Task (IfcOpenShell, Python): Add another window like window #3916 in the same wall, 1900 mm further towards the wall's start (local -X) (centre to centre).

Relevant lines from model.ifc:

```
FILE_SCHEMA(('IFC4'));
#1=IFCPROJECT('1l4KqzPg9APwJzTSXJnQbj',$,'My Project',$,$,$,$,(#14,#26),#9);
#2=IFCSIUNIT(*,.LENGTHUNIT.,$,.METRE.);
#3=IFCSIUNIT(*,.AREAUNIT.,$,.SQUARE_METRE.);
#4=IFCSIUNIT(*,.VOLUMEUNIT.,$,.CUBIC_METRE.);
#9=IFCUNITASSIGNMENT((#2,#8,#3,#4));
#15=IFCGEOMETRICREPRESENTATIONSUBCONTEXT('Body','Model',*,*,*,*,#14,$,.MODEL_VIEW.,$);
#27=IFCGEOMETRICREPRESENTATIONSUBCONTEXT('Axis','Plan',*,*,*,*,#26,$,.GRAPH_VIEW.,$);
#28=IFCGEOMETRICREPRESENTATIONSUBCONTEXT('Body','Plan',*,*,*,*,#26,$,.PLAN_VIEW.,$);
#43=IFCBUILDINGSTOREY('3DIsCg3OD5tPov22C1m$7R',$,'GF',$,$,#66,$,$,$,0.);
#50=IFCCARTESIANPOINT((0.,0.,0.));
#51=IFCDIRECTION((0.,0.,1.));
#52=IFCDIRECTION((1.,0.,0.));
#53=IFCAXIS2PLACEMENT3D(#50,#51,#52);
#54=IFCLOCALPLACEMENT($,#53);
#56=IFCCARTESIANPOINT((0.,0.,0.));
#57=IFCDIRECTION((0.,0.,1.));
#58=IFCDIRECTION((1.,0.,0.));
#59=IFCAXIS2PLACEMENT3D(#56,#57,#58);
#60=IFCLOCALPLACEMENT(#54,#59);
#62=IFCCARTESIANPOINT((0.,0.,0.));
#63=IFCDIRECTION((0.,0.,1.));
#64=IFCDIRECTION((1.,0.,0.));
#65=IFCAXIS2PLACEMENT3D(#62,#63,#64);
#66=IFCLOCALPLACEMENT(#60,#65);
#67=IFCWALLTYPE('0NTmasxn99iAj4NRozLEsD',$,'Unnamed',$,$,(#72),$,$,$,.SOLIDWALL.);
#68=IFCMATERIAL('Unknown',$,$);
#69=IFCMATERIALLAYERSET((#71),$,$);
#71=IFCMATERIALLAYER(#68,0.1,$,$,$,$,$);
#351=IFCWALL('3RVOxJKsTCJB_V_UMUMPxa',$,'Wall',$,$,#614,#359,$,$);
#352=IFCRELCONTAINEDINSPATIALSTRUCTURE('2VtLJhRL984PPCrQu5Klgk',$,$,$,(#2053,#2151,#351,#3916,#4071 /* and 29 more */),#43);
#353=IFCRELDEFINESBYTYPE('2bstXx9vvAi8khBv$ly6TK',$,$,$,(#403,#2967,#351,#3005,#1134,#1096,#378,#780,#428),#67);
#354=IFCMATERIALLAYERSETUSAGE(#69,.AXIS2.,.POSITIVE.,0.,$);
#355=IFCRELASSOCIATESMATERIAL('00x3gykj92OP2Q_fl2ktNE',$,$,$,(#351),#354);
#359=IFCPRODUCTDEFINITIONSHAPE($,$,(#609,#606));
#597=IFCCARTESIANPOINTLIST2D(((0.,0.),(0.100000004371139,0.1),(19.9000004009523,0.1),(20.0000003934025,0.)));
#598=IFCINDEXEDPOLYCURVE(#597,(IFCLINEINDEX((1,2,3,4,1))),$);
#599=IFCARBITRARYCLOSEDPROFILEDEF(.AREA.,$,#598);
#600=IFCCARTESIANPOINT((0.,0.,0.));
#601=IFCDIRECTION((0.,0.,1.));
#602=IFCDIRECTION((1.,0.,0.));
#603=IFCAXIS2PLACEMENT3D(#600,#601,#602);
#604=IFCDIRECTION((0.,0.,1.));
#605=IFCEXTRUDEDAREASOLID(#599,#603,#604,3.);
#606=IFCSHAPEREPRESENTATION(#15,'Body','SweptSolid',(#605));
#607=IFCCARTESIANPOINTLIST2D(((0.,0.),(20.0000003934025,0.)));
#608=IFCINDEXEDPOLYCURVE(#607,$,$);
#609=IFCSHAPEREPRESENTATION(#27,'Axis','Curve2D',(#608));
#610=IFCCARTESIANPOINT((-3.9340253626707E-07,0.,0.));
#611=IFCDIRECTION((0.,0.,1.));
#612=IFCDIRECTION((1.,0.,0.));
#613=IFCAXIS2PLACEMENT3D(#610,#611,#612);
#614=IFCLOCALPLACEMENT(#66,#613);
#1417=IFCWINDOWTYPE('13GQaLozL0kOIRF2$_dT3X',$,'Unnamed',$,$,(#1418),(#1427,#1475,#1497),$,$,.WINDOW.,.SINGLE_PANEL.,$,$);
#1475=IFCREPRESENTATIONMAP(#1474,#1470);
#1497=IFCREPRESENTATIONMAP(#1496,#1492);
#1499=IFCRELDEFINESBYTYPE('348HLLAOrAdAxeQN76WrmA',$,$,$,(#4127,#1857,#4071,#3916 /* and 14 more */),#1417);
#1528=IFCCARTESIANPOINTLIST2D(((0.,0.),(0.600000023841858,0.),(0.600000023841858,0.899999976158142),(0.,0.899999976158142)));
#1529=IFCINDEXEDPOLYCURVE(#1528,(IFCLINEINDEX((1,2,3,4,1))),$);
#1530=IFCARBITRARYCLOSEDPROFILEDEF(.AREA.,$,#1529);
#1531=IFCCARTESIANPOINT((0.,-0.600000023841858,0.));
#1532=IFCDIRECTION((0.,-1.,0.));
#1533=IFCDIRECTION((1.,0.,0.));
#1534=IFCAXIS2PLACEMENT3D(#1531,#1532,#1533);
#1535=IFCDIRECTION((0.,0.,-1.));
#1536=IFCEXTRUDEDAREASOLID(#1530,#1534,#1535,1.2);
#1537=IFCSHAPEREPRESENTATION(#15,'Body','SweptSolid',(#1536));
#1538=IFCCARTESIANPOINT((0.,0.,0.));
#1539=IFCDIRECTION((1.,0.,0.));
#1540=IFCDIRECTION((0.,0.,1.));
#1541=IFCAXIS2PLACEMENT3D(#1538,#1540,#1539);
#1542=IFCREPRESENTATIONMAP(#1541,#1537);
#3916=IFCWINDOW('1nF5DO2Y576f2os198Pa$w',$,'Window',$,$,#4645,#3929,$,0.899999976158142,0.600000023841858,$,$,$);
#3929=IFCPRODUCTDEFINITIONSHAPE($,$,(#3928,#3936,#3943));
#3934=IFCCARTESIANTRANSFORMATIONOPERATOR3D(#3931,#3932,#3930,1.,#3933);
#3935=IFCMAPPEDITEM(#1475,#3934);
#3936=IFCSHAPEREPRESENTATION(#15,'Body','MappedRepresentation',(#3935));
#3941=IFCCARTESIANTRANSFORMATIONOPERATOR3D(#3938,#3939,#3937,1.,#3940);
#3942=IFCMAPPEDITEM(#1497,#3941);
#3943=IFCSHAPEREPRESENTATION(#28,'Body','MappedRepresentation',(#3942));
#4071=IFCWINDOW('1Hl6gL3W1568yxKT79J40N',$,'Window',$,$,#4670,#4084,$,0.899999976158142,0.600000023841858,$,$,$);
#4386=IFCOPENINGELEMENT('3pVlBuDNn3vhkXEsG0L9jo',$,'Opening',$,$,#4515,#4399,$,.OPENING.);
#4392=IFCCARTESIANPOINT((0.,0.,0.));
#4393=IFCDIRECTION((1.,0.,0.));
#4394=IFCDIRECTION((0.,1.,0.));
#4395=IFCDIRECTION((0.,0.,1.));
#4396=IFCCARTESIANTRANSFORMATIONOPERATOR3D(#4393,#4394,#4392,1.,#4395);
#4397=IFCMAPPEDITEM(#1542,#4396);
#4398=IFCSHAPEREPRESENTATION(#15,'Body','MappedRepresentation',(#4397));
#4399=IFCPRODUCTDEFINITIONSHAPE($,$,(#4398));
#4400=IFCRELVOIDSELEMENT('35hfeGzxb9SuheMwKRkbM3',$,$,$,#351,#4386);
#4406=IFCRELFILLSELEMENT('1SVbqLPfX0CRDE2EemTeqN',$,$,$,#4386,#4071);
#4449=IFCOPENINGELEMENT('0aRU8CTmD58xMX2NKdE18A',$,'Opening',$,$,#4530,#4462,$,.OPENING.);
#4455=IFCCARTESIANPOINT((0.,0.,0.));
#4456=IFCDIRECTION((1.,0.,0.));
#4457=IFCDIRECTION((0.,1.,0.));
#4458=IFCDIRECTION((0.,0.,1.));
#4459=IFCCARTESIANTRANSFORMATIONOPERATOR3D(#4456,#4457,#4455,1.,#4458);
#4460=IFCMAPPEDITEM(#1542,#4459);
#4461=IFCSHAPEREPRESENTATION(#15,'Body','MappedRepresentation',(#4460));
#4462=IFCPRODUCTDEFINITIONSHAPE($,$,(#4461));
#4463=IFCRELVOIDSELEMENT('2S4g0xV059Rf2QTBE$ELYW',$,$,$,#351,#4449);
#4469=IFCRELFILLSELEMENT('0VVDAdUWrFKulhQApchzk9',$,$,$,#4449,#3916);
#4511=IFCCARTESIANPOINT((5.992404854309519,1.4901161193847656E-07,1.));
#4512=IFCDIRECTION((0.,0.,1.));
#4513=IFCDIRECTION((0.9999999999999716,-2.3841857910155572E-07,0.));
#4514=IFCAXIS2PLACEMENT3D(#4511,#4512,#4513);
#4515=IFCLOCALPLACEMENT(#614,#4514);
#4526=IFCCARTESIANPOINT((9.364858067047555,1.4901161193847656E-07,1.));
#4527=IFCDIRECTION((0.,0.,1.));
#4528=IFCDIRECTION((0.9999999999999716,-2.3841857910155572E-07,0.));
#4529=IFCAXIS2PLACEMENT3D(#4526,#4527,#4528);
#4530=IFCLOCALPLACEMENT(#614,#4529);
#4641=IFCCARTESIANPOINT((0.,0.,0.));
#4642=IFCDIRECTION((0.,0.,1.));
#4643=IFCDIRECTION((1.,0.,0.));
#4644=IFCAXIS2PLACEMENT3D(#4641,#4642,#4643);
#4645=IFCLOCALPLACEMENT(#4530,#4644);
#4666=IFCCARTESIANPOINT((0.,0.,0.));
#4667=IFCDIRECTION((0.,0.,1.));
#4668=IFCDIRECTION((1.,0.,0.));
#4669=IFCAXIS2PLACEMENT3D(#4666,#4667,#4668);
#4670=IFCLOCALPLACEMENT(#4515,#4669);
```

```python
import ifcopenshell
import ifcopenshell.api.feature
import ifcopenshell.api.geometry
import ifcopenshell.api.root
import ifcopenshell.geom
import ifcopenshell.util.element
import ifcopenshell.util.placement
import ifcopenshell.util.shape
import ifcopenshell.util.unit

model = ifcopenshell.open("model.ifc")
unit_scale = ifcopenshell.util.unit.calculate_unit_scale(model)
settings = ifcopenshell.geom.settings()


def volume(element):
    """Net volume in cubic metres, openings subtracted."""
    shape = ifcopenshell.geom.create_shape(settings, element)
    return ifcopenshell.util.shape.get_volume(shape.geometry)


window = model.by_guid("1nF5DO2Y576f2os198Pa$w")
opening = window.FillsVoids[0].RelatingOpeningElement
wall = opening.VoidsElements[0].RelatingBuildingElement
before = volume(wall)
shift = ifcopenshell.util.placement.get_local_placement(wall.ObjectPlacement)[:3, 0] * -1.9 / unit_scale

# copy_class copies the void relationship, type, container and properties, but no geometry.
new_opening = ifcopenshell.api.root.copy_class(model, product=opening)
new_opening.Representation = ifcopenshell.util.element.copy_deep(
    model, opening.Representation, exclude=["IfcGeometricRepresentationContext", "IfcRepresentationMap"]
)
new_window = ifcopenshell.api.root.copy_class(model, product=window)
new_window.Representation = ifcopenshell.util.element.copy_deep(
    model, window.Representation, exclude=["IfcGeometricRepresentationContext", "IfcRepresentationMap"]
)
ifcopenshell.api.feature.add_filling(model, opening=new_opening, element=new_window)

for old, new in ((opening, new_opening), (window, new_window)):
    matrix = ifcopenshell.util.placement.get_local_placement(old.ObjectPlacement)
    matrix[:3, 3] += shift
    ifcopenshell.api.geometry.edit_object_placement(model, product=new, matrix=matrix, is_si=False)

after = volume(wall)

print(f"wall volume {before:.3f} -> {after:.3f} m3")

model.write("model_v2.ifc")
```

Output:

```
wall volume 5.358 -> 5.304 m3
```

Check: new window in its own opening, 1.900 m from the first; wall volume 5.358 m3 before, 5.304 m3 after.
